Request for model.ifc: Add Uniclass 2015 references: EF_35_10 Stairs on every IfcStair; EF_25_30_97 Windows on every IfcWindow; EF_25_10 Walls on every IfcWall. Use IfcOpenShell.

First a look at what the model holds.

```python
import ifcopenshell

model = ifcopenshell.open("model.ifc")
print(model.schema)
print("classifications:", [c.Name for c in model.by_type("IfcClassification")])
for ifc_class in ("IfcDoor", "IfcRoof", "IfcStair", "IfcWall", "IfcWindow"):
    print(ifc_class, len(model.by_type(ifc_class)))
```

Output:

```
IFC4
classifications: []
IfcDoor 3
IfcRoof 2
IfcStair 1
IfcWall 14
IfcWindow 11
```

```python
import ifcopenshell
import ifcopenshell.api.classification

model = ifcopenshell.open("model.ifc")

system = ifcopenshell.api.classification.add_classification(model, classification="Uniclass 2015")

codes = {
    "IfcStair": ("EF_35_10", "Stairs"),
    "IfcWindow": ("EF_25_30_97", "Windows"),
    "IfcWall": ("EF_25_10", "Walls"),
}
for ifc_class, (code, name) in codes.items():
    products = model.by_type(ifc_class)
    ifcopenshell.api.classification.add_reference(
        model, products=products, classification=system, identification=code, name=name
    )
    print(code, len(products))

model.write("model-out.ifc")
```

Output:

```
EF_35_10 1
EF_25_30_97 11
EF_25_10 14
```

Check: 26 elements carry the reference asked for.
